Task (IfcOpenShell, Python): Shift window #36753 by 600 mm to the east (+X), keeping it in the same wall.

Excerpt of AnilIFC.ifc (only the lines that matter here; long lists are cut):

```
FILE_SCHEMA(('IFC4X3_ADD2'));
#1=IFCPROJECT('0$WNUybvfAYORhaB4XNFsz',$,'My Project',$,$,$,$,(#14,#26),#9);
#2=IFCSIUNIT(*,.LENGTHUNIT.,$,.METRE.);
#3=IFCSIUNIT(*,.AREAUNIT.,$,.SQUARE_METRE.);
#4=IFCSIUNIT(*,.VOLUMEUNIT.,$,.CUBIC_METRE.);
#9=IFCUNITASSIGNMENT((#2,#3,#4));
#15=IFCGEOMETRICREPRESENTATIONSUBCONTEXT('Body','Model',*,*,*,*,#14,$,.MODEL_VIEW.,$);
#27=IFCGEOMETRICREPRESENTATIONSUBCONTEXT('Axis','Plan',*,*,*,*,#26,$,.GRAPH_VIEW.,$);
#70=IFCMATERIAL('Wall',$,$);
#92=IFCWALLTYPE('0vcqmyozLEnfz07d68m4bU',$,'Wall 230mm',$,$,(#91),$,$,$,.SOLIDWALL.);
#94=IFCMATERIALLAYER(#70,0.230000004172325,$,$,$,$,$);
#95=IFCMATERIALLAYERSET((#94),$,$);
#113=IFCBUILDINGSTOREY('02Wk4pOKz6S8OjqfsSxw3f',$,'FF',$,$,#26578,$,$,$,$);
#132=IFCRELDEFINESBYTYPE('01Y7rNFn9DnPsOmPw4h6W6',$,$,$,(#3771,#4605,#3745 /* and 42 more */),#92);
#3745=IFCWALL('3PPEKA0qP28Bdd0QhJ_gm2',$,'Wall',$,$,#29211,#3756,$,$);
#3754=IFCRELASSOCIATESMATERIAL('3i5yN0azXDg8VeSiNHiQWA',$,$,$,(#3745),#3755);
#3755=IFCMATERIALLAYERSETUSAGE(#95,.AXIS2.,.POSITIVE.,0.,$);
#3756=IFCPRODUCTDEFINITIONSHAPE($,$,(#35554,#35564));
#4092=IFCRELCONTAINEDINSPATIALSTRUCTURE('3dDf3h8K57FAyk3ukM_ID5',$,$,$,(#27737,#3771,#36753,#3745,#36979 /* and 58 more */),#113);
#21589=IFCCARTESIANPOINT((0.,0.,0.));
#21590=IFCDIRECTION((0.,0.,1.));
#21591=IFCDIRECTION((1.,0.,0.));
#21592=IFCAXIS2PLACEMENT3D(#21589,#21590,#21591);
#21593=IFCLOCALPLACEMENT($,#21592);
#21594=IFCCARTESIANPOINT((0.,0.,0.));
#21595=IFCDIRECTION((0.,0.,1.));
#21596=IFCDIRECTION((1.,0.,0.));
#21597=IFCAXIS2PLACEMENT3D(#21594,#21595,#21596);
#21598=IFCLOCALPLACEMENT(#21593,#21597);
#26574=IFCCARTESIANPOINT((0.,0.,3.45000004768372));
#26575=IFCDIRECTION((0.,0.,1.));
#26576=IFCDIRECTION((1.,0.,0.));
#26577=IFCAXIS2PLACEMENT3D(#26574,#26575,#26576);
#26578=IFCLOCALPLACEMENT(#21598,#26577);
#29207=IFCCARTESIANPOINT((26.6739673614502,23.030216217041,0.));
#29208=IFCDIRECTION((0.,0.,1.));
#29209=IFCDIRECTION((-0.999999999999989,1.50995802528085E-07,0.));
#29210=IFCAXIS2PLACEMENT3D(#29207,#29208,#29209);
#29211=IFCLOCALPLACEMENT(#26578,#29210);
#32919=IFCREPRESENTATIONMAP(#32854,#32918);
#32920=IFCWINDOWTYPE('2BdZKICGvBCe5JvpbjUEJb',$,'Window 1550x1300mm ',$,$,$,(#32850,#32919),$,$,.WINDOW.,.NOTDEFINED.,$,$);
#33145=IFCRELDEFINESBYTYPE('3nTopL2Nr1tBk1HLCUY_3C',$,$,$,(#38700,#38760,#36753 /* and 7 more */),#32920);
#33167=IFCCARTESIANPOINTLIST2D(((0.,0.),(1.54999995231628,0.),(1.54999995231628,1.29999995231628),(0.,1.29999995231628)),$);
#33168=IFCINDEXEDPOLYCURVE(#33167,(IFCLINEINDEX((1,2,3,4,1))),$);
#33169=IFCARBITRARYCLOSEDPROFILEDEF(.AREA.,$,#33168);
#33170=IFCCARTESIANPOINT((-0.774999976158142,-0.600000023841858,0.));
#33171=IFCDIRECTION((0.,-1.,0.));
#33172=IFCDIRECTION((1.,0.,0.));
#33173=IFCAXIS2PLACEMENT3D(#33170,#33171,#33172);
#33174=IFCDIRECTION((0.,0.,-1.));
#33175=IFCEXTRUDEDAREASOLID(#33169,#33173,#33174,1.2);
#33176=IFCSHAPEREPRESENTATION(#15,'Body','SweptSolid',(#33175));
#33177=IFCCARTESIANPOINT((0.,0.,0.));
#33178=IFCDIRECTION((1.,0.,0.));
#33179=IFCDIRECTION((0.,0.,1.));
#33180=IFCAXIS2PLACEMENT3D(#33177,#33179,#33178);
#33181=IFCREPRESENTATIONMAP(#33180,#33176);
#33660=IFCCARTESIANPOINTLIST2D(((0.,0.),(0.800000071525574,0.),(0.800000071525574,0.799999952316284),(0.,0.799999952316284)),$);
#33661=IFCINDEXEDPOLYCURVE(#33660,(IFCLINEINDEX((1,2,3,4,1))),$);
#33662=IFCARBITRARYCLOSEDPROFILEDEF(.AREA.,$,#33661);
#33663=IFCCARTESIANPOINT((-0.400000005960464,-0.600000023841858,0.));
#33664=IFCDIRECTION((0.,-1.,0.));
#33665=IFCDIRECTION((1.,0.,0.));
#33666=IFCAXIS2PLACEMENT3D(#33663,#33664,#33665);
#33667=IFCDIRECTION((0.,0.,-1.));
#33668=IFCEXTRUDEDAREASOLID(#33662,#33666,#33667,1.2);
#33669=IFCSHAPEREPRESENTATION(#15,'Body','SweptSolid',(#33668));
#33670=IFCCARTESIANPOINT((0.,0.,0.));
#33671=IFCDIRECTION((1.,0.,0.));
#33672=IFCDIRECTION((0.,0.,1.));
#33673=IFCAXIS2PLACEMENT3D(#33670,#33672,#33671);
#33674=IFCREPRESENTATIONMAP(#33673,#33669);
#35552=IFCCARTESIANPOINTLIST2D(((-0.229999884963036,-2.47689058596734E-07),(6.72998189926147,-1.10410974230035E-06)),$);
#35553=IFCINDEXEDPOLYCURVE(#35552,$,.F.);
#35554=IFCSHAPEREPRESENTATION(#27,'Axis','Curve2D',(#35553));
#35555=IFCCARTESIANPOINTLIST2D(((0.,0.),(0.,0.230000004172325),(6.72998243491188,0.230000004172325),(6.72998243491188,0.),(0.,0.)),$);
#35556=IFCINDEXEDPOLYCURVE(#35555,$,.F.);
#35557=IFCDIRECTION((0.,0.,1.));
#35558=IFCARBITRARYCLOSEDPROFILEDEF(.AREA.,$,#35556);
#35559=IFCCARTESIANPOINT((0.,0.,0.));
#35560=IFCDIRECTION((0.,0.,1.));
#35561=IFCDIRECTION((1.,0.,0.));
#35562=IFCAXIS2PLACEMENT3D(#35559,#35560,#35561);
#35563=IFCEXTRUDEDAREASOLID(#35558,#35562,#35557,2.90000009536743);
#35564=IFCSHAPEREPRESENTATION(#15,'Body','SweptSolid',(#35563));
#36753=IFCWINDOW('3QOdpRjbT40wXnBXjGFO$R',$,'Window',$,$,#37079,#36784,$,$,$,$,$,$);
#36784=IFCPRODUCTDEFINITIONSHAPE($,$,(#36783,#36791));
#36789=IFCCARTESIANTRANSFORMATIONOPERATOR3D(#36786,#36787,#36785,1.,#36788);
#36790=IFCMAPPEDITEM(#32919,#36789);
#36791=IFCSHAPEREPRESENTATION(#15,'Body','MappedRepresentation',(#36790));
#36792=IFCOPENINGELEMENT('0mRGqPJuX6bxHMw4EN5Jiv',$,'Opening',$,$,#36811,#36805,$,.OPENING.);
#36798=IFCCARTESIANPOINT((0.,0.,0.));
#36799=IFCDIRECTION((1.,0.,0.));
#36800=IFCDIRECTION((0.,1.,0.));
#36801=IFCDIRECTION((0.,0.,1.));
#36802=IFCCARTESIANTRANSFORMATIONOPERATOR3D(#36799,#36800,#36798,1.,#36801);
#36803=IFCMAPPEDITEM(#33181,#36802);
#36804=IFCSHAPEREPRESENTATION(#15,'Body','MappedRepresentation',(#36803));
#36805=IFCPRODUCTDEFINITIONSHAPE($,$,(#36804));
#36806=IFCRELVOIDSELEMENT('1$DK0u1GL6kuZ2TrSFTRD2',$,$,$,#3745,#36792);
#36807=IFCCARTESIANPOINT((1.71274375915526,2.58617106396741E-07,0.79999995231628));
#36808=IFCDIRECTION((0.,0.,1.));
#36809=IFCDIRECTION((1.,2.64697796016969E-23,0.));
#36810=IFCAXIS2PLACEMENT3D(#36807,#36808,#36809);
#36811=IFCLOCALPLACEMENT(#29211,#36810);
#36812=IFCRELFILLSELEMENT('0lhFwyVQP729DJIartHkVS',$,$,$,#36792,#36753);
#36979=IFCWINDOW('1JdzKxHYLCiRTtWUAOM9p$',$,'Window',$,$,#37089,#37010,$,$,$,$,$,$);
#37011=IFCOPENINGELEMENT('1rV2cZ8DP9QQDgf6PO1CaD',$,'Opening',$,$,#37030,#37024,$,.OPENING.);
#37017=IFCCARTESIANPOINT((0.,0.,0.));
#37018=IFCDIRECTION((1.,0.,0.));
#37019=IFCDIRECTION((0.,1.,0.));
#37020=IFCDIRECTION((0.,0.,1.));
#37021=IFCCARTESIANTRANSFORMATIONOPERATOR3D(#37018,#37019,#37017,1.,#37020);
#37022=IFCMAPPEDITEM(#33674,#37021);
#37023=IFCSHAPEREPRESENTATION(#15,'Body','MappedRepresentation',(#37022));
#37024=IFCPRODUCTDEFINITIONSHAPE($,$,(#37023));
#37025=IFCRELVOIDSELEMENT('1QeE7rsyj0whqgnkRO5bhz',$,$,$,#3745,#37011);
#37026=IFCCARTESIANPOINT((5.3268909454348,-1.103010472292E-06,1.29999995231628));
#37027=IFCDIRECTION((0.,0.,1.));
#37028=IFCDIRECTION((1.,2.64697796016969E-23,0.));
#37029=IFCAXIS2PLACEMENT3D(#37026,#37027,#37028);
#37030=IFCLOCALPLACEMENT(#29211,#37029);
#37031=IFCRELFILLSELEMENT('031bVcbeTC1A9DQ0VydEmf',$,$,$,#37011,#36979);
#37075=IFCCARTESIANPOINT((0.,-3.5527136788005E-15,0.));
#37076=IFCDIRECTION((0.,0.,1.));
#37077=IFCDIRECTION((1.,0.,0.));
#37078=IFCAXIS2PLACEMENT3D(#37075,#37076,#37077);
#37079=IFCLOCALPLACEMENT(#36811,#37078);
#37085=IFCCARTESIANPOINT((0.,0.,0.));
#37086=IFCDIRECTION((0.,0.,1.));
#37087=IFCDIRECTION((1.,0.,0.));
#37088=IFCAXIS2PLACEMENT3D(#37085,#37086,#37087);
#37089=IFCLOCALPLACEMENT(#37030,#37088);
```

```python
import ifcopenshell
import ifcopenshell.api.geometry
import ifcopenshell.util.placement

model = ifcopenshell.open("AnilIFC.ifc")

window = model.by_guid("3QOdpRjbT40wXnBXjGFO$R")
opening = window.FillsVoids[0].RelatingOpeningElement
wall = opening.VoidsElements[0].RelatingBuildingElement

wall_matrix = ifcopenshell.util.placement.get_local_placement(wall.ObjectPlacement)
shift = wall_matrix[:3, 0] * -0.6
before = ifcopenshell.util.placement.get_local_placement(window.ObjectPlacement)[:3, 3].copy()

# The window is placed relative to its opening, so it follows when the opening moves.
matrix = ifcopenshell.util.placement.get_local_placement(opening.ObjectPlacement)
matrix[:3, 3] += shift
ifcopenshell.api.geometry.edit_object_placement(
    model, product=opening, matrix=matrix, is_si=False, should_transform_children=True
)

after = ifcopenshell.util.placement.get_local_placement(window.ObjectPlacement)[:3, 3]
print("window moved by", (after - before).round(3) + 0.0)

model.write("AnilIFC_v2.ifc")
```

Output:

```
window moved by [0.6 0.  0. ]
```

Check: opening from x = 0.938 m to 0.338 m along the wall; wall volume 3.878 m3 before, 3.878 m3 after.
